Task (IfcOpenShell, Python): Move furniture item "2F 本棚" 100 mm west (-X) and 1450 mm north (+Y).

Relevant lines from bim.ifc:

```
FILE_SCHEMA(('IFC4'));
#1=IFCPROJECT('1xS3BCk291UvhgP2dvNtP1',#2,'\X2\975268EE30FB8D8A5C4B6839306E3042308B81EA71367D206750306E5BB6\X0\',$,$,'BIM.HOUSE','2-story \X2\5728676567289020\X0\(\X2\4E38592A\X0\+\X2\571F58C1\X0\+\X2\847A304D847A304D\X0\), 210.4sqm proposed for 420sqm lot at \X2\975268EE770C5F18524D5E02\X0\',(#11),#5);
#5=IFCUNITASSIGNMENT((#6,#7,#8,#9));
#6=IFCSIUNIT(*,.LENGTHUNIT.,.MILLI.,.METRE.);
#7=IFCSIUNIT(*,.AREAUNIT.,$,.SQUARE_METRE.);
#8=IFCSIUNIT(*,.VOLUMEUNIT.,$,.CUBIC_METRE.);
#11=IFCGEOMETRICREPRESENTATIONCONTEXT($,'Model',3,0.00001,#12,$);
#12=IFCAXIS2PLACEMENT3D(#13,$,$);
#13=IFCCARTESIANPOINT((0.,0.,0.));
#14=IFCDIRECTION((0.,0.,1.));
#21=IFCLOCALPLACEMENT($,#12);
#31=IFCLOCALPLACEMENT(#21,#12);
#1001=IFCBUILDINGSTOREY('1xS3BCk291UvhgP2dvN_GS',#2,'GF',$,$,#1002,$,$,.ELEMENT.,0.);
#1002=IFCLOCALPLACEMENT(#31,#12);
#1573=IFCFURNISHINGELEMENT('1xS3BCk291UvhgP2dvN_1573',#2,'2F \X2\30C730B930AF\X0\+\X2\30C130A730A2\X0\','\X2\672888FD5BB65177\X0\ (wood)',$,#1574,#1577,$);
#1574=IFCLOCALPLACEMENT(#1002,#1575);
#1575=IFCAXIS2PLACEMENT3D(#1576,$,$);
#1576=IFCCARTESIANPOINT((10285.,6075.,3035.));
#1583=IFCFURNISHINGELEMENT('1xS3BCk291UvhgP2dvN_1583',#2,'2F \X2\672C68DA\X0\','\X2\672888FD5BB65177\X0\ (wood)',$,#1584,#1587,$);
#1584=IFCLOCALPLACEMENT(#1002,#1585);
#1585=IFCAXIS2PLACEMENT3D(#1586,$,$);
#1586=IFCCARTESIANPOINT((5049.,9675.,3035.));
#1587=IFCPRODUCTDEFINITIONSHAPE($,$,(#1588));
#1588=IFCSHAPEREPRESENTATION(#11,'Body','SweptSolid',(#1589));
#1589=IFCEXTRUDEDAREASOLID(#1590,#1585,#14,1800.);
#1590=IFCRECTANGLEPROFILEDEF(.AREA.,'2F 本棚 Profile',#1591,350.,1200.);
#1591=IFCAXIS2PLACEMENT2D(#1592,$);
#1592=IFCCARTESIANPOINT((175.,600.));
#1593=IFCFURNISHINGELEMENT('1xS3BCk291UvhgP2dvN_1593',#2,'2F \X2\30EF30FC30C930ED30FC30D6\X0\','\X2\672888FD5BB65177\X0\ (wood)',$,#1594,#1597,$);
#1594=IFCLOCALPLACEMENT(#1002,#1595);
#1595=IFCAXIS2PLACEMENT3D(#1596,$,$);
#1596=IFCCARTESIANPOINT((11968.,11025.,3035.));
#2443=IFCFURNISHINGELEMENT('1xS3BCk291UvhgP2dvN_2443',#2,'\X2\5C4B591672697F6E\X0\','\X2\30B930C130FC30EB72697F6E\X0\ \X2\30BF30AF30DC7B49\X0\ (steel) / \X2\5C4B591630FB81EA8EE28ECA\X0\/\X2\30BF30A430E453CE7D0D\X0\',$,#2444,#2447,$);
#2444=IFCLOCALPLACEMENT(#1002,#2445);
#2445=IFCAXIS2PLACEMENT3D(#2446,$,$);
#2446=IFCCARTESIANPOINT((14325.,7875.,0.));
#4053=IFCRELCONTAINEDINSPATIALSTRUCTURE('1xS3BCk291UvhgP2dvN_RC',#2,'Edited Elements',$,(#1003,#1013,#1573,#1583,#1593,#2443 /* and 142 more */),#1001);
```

```python
import ifcopenshell
import ifcopenshell.api.geometry
import ifcopenshell.util.placement

model = ifcopenshell.open("bim.ifc")

item = model.by_id(1583)
matrix = ifcopenshell.util.placement.get_local_placement(item.ObjectPlacement)
matrix[0, 3] -= 100.0
matrix[1, 3] += 1450.0
ifcopenshell.api.geometry.edit_object_placement(model, product=item, matrix=matrix, is_si=False)

print(ifcopenshell.util.placement.get_local_placement(item.ObjectPlacement).round(3) + 0.0)

model.write("bim_updated.ifc")
```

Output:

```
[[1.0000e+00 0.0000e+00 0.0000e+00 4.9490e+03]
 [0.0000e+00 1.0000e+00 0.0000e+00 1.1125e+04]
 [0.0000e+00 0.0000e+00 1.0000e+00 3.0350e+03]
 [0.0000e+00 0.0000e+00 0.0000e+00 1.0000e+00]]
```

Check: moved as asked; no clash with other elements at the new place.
